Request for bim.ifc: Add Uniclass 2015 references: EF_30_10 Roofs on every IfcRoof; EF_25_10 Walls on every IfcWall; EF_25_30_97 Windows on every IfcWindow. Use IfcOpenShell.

First a look at what the model holds.

```python
import ifcopenshell

model = ifcopenshell.open("bim.ifc")
print(model.schema)
print("classifications:", [c.Name for c in model.by_type("IfcClassification")])
for ifc_class in ("IfcDoor", "IfcRoof", "IfcStair", "IfcWall", "IfcWindow"):
    print(ifc_class, len(model.by_type(ifc_class)))
```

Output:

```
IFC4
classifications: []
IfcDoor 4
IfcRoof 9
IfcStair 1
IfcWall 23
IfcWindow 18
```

```python
import ifcopenshell
import ifcopenshell.api.classification

model = ifcopenshell.open("bim.ifc")

system = ifcopenshell.api.classification.add_classification(model, classification="Uniclass 2015")

codes = {
    "IfcRoof": ("EF_30_10", "Roofs"),
    "IfcWall": ("EF_25_10", "Walls"),
    "IfcWindow": ("EF_25_30_97", "Windows"),
}
for ifc_class, (code, name) in codes.items():
    products = model.by_type(ifc_class)
    ifcopenshell.api.classification.add_reference(
        model, products=products, classification=system, identification=code, name=name
    )
    print(code, len(products))

model.write("bim-out.ifc")
```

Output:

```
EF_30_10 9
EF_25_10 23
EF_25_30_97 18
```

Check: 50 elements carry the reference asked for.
